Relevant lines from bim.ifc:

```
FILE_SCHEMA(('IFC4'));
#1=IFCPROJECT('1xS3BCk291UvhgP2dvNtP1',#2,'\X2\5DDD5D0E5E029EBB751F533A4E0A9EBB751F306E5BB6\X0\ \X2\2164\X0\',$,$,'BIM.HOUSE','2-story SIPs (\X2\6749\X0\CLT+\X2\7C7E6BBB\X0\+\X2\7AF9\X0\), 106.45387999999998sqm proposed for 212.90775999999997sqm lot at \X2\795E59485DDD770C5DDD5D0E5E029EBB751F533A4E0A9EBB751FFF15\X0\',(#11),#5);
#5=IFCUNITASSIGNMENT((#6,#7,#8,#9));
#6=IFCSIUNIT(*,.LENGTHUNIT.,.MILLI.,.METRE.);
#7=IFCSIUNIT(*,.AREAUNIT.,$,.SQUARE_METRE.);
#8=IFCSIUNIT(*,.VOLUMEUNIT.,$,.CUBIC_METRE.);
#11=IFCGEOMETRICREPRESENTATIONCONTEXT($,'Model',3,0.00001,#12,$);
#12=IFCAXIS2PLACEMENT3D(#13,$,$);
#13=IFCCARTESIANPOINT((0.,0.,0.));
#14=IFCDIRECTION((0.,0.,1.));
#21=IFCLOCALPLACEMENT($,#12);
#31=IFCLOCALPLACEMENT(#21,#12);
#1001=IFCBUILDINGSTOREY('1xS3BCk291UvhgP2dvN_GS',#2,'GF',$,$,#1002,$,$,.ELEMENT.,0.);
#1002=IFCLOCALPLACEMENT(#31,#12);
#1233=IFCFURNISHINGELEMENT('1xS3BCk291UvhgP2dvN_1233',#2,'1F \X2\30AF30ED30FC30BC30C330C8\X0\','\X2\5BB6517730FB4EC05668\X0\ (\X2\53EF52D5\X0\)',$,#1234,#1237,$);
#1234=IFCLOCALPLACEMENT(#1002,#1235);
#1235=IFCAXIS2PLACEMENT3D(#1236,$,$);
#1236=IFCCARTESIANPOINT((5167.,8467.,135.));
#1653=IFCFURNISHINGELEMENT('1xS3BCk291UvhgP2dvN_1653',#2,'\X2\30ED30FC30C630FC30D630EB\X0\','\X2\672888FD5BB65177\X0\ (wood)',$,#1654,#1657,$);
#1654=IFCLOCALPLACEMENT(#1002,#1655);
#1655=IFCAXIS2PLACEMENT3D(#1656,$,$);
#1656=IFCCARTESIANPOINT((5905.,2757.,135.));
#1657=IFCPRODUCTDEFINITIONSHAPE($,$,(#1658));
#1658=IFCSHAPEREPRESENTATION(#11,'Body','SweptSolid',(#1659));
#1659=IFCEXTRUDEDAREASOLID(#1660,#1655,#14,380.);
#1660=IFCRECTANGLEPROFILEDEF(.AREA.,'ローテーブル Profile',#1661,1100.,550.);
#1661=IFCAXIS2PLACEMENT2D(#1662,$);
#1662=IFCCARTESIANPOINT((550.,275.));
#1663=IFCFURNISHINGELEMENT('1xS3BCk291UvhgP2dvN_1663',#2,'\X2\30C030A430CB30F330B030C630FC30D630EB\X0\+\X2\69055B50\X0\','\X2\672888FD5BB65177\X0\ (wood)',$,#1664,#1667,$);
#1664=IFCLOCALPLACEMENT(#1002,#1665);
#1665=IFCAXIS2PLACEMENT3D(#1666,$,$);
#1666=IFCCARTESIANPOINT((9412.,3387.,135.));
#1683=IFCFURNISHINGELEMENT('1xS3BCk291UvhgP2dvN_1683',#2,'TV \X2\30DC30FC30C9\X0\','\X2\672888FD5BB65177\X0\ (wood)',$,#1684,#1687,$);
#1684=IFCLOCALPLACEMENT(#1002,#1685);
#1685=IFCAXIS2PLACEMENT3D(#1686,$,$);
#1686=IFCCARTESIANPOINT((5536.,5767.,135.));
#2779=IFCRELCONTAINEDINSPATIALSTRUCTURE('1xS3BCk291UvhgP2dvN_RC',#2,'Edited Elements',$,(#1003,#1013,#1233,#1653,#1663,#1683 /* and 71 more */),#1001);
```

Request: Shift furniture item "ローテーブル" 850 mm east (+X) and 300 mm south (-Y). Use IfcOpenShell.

```python
import ifcopenshell
import ifcopenshell.api.geometry
import ifcopenshell.util.placement
import ifcopenshell.util.unit

model = ifcopenshell.open("bim.ifc")
unit_scale = ifcopenshell.util.unit.calculate_unit_scale(model)

item = model.by_guid("1xS3BCk291UvhgP2dvN_1653")
matrix = ifcopenshell.util.placement.get_local_placement(item.ObjectPlacement)
matrix[0, 3] += 0.85 / unit_scale
matrix[1, 3] -= 0.3 / unit_scale
ifcopenshell.api.geometry.edit_object_placement(model, product=item, matrix=matrix, is_si=False)

print(ifcopenshell.util.placement.get_local_placement(item.ObjectPlacement).round(3) + 0.0)

model.write("bim_rev.ifc")
```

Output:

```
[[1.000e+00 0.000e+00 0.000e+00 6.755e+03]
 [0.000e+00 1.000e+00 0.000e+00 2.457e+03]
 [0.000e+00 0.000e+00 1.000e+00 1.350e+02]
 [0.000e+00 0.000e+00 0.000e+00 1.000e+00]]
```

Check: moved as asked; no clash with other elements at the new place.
